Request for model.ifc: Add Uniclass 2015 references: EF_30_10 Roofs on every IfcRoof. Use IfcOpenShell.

First a look at what the model holds.

```python
import ifcopenshell

model = ifcopenshell.open("model.ifc")
print(model.schema)
print("classifications:", [c.Name for c in model.by_type("IfcClassification")])
for ifc_class in ("IfcDoor", "IfcRoof", "IfcStair", "IfcWall", "IfcWindow"):
    print(ifc_class, len(model.by_type(ifc_class)))
```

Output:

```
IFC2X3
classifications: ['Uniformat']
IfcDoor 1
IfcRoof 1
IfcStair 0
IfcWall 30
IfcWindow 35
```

```python
import ifcopenshell
import ifcopenshell.api.classification

model = ifcopenshell.open("model.ifc")

# IFC2X3 requires Source and Edition and has no link from the project to the system.
system = model.create_entity("IfcClassification", Source="NBS", Edition="2015", Name="Uniclass 2015")

codes = {
    "IfcRoof": ("EF_30_10", "Roofs"),
}
for ifc_class, (code, name) in codes.items():
    products = model.by_type(ifc_class)
    ifcopenshell.api.classification.add_reference(
        model, products=products, classification=system, identification=code, name=name
    )
    print(code, len(products))

model.write("model_rev.ifc")
```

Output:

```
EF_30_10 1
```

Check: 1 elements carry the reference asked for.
